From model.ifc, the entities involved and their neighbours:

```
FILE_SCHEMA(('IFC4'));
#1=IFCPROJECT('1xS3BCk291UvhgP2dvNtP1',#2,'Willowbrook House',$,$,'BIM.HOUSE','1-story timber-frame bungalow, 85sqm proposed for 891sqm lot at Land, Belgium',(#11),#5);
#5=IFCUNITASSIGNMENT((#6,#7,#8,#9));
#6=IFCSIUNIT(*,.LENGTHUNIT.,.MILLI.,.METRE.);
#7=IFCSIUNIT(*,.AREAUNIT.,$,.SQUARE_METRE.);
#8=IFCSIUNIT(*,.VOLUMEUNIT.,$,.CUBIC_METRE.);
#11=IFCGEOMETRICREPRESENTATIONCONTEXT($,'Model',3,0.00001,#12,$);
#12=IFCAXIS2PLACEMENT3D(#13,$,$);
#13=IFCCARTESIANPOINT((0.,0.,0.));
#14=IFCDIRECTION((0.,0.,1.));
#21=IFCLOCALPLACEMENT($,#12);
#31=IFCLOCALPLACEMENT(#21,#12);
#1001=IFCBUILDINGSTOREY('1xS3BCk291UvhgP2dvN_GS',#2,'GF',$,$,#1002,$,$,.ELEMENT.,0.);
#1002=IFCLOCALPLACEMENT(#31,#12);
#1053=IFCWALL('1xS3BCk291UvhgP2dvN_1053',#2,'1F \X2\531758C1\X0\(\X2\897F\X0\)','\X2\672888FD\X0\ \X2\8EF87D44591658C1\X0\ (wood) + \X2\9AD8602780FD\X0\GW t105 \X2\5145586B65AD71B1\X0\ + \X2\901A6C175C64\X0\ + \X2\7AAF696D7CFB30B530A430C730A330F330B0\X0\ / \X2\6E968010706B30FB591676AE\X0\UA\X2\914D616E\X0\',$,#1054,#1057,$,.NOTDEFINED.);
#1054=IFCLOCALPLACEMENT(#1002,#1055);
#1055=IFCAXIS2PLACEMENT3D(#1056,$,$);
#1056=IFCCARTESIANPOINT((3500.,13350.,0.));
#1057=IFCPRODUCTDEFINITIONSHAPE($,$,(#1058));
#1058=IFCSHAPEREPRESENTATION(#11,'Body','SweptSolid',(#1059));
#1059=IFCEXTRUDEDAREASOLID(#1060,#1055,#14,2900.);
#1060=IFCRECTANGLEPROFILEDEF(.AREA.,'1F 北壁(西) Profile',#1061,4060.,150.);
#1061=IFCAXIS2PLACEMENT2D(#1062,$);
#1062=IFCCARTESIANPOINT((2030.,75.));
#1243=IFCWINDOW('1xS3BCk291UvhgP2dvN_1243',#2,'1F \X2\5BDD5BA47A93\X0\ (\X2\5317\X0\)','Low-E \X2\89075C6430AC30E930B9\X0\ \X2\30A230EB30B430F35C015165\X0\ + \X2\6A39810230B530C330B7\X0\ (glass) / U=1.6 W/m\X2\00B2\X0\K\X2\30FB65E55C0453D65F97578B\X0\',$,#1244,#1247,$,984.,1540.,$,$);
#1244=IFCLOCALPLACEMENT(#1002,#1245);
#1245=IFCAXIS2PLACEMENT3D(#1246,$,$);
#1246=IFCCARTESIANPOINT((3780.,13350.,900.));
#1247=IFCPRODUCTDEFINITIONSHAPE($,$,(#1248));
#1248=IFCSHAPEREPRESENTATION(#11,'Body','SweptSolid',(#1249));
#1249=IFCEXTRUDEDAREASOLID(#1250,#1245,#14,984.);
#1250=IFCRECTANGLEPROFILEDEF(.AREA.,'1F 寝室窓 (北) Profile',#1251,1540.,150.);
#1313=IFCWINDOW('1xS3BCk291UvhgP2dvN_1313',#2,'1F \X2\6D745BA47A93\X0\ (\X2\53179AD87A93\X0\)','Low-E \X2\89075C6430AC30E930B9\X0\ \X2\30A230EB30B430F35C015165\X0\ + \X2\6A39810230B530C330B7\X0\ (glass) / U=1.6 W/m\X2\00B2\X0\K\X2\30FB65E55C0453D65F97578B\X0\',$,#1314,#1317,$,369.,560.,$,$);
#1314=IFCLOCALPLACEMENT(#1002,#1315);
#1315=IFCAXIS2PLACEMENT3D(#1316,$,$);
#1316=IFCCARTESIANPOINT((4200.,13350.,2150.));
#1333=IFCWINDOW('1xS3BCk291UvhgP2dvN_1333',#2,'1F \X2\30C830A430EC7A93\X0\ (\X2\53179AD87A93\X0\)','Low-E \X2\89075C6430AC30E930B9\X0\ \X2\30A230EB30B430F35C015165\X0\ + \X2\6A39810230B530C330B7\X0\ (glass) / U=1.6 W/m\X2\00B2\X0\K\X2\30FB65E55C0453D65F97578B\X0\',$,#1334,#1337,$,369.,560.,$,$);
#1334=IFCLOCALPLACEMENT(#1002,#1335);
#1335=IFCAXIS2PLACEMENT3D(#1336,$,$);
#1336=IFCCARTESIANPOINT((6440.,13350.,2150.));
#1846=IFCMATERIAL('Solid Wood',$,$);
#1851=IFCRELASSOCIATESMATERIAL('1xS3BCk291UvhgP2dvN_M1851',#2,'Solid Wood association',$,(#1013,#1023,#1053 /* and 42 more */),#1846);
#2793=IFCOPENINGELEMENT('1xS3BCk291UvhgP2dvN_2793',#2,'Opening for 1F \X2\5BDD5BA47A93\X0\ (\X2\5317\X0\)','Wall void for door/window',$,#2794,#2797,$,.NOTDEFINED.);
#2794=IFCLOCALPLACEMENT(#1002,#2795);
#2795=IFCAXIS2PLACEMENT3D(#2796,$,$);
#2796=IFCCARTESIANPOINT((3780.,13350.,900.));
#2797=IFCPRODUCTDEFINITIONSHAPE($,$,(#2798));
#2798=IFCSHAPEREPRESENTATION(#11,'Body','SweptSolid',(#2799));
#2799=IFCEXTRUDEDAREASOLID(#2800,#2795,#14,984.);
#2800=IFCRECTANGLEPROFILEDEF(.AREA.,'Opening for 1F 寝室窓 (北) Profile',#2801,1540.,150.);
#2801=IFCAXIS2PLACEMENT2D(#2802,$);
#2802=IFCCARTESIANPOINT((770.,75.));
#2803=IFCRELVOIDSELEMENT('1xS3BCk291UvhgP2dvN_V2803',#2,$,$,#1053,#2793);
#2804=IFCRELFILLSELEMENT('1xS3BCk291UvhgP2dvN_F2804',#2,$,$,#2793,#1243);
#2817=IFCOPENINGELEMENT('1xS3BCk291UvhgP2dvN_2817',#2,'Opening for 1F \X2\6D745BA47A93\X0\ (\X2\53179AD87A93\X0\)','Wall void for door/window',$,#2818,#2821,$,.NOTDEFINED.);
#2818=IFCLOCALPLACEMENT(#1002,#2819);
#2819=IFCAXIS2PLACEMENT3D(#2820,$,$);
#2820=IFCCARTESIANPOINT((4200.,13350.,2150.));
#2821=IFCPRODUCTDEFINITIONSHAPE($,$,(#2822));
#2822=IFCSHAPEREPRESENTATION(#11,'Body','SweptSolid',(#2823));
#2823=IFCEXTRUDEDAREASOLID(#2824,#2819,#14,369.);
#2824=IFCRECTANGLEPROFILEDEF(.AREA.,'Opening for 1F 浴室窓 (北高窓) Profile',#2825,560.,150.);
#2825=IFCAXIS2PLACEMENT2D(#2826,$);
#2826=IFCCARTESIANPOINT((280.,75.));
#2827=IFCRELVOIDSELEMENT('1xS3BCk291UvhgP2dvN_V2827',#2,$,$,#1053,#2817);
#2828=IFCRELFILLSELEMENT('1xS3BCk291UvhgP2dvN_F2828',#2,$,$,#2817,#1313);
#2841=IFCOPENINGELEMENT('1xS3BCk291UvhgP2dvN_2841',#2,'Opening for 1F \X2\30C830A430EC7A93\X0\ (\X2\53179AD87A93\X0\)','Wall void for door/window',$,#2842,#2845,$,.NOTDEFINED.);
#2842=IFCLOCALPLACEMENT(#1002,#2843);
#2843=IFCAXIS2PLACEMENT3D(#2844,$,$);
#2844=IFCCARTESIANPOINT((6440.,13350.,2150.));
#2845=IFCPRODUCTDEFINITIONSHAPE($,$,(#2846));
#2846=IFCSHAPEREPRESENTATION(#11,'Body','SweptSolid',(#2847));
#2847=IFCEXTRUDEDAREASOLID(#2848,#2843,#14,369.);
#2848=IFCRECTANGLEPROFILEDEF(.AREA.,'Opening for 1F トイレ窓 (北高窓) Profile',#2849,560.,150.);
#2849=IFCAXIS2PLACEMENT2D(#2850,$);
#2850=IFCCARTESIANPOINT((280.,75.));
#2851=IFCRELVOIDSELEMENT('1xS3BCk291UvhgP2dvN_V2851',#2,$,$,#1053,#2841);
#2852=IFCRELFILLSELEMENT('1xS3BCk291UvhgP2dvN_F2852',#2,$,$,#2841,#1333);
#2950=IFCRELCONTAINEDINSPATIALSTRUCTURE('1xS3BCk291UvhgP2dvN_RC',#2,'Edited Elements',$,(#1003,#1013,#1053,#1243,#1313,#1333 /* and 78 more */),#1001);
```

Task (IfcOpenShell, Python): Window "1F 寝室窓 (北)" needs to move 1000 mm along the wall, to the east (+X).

```python
import ifcopenshell
import ifcopenshell.api.geometry
import ifcopenshell.util.placement
import ifcopenshell.util.unit

model = ifcopenshell.open("model.ifc")
unit_scale = ifcopenshell.util.unit.calculate_unit_scale(model)

window = model.by_guid("1xS3BCk291UvhgP2dvN_1243")
opening = window.FillsVoids[0].RelatingOpeningElement
wall = opening.VoidsElements[0].RelatingBuildingElement

wall_matrix = ifcopenshell.util.placement.get_local_placement(wall.ObjectPlacement)
shift = wall_matrix[:3, 0] * 1 / unit_scale
before = ifcopenshell.util.placement.get_local_placement(window.ObjectPlacement)[:3, 3].copy()

# The window is not placed relative to its opening, so move both.
for product in (opening, window):
    matrix = ifcopenshell.util.placement.get_local_placement(product.ObjectPlacement)
    matrix[:3, 3] += shift
    ifcopenshell.api.geometry.edit_object_placement(model, product=product, matrix=matrix, is_si=False)

after = ifcopenshell.util.placement.get_local_placement(window.ObjectPlacement)[:3, 3]
print("window moved by", (after - before).round(3) + 0.0)

model.write("model_edited.ifc")
```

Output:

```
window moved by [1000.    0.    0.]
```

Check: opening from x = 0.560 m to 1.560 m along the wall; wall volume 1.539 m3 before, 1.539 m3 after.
